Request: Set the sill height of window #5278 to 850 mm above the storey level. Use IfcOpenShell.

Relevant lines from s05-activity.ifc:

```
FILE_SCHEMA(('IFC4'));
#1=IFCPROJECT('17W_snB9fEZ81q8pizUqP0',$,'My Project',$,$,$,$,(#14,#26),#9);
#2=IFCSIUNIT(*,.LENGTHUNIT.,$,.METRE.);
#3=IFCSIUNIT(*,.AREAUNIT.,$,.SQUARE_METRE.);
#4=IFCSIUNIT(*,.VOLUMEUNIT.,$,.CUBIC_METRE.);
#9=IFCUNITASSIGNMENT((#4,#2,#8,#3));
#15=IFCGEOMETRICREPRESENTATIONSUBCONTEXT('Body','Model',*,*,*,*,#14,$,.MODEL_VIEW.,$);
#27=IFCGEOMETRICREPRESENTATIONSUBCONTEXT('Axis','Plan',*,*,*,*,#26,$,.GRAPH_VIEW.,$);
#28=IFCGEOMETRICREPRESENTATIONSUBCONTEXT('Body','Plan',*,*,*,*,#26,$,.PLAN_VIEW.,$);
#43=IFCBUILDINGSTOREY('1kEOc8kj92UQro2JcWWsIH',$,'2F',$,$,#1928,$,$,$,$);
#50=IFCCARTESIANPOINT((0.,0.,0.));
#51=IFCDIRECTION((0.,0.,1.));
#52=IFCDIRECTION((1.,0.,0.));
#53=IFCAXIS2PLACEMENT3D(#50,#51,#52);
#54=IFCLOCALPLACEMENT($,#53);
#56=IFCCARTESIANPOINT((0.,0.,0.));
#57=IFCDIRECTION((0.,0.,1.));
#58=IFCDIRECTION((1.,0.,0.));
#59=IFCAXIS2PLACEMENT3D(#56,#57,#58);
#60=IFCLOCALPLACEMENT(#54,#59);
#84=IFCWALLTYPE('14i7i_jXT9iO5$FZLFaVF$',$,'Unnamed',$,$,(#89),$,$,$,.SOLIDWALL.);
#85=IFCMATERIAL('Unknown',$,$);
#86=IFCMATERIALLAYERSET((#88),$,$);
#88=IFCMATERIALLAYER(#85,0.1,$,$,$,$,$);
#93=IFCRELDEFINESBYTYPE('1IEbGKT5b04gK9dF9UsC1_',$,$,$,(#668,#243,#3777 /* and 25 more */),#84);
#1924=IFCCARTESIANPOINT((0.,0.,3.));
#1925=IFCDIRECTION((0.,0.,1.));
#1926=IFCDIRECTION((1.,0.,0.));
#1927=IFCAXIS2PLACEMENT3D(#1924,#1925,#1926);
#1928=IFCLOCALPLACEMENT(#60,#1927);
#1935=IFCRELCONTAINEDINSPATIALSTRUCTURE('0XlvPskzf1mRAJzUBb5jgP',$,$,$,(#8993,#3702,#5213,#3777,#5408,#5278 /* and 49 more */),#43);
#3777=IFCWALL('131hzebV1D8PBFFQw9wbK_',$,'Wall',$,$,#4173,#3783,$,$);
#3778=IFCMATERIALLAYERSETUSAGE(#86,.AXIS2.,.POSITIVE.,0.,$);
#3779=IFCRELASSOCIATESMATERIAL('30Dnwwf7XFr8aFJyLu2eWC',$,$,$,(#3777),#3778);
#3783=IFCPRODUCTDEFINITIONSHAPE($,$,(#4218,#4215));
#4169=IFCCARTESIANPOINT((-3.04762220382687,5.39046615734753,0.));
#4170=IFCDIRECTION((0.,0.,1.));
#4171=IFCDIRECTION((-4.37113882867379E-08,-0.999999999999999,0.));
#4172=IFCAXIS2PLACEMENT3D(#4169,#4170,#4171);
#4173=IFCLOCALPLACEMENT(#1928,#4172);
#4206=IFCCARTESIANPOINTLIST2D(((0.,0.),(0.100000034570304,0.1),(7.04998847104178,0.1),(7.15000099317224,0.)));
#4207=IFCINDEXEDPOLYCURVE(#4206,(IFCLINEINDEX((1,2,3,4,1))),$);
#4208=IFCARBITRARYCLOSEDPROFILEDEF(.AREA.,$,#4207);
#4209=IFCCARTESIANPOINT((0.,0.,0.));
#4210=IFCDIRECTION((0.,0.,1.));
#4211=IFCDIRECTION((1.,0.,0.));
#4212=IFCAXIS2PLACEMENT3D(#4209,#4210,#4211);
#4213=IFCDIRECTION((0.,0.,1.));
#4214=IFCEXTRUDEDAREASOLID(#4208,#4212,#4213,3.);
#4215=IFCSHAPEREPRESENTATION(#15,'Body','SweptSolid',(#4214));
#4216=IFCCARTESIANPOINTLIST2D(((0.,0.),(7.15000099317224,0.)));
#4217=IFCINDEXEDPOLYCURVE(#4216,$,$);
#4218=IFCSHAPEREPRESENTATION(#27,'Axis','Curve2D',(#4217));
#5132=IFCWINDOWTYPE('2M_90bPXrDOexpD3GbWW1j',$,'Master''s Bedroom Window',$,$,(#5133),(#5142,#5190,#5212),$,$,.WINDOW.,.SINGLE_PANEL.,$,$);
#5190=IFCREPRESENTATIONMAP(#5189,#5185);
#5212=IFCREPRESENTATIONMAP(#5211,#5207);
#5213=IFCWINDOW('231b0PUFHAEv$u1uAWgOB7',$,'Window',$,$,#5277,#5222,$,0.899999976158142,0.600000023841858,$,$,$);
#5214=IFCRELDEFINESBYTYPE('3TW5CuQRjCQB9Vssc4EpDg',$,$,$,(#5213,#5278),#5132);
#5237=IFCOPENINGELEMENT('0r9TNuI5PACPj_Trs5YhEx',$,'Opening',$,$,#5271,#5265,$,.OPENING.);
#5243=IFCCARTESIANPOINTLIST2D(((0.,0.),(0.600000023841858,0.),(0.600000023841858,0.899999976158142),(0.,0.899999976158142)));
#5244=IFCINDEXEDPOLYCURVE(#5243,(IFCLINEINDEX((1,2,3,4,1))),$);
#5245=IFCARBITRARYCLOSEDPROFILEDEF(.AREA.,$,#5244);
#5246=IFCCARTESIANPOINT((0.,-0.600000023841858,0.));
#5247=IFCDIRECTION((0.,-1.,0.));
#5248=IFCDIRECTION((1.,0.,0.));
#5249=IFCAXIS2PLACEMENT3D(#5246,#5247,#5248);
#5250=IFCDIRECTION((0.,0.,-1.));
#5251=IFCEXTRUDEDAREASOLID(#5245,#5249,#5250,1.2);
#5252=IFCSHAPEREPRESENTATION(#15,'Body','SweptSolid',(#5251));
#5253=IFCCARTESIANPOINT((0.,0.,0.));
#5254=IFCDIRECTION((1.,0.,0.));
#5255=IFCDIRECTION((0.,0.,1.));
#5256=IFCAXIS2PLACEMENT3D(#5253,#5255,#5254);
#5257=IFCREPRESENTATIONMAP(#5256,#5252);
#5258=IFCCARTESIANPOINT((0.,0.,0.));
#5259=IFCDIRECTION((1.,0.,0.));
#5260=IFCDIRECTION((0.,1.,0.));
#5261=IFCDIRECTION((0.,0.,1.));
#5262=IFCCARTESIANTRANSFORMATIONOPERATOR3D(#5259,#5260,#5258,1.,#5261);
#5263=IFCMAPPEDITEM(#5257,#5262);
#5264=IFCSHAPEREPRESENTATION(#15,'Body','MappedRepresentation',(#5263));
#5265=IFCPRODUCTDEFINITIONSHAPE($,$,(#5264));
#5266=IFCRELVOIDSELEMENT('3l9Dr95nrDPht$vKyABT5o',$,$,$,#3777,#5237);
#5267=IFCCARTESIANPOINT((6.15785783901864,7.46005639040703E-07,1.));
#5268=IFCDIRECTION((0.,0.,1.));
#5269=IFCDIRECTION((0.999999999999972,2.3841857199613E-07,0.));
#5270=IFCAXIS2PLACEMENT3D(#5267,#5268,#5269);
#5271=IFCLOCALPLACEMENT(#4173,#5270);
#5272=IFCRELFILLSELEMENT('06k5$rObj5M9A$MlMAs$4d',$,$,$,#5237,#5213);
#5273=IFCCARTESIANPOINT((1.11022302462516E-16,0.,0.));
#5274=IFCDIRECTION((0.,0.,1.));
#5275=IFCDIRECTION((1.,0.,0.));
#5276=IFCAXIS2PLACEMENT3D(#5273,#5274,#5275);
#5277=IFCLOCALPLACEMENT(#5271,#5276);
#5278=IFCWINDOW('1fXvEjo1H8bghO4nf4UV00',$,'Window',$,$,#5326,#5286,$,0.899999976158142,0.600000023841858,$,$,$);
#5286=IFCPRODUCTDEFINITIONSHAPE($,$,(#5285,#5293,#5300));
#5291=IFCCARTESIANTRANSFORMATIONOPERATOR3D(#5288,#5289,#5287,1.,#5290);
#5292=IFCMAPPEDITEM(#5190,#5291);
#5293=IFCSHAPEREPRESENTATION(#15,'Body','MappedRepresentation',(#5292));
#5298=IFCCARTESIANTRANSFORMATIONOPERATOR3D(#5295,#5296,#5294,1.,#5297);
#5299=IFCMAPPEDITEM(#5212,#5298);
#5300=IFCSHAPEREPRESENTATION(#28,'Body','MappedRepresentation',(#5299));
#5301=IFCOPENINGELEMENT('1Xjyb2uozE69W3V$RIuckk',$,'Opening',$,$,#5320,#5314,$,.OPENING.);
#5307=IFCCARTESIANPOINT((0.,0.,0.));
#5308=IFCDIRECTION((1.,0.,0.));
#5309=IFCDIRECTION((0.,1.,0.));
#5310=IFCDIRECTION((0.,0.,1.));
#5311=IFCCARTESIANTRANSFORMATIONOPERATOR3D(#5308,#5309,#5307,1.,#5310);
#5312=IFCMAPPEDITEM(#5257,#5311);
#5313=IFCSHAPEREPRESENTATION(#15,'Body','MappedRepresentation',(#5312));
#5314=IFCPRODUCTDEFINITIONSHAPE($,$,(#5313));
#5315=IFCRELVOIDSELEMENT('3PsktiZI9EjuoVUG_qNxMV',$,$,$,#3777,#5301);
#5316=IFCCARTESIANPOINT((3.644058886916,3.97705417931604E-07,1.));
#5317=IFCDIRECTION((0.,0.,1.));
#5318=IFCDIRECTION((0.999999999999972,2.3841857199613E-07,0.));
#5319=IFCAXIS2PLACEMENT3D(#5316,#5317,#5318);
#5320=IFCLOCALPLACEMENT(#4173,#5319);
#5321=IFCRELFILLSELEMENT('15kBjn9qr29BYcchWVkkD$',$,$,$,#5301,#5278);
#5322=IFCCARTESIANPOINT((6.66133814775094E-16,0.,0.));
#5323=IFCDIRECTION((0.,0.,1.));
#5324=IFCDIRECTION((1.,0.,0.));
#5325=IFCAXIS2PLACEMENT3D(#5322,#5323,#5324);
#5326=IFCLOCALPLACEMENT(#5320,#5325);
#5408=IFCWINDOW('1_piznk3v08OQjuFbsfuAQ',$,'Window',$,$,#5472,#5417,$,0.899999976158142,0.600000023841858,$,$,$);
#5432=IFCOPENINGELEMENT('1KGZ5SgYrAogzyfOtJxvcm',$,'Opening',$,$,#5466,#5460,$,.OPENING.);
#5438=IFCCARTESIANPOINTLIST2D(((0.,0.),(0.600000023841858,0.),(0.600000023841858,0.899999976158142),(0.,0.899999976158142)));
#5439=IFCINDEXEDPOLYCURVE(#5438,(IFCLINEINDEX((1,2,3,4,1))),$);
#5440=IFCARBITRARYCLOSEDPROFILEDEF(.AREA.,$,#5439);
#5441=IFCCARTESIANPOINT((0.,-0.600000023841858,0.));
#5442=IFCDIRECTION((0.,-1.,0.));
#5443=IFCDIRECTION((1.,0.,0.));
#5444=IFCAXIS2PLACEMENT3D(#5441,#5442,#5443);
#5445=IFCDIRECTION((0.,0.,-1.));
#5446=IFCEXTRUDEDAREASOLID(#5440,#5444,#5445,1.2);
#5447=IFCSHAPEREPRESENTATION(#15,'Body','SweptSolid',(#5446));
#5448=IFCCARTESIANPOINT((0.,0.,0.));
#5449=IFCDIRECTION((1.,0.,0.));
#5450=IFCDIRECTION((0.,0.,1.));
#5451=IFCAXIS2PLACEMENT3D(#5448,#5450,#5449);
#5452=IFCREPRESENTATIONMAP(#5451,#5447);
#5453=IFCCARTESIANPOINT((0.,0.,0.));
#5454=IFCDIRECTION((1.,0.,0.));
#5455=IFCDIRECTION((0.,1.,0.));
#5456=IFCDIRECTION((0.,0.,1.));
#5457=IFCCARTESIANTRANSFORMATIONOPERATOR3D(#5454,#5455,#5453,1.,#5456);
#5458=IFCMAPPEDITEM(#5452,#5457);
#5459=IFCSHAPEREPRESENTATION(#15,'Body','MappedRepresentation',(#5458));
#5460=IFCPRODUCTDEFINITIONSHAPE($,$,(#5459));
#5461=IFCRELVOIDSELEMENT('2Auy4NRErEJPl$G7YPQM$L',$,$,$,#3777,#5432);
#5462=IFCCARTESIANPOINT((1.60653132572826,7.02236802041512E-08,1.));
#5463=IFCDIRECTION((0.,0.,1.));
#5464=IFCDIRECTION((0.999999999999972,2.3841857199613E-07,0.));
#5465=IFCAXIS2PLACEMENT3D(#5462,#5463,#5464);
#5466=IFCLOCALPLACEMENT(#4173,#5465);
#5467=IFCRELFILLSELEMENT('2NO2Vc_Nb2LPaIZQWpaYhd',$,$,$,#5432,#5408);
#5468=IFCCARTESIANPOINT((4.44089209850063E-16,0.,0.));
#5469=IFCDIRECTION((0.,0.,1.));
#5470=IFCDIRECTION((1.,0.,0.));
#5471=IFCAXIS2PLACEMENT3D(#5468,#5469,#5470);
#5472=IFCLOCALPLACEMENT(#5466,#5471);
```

```python
import numpy as np
import ifcopenshell
import ifcopenshell.api.geometry
import ifcopenshell.geom
import ifcopenshell.util.element
import ifcopenshell.util.placement
import ifcopenshell.util.shape
import ifcopenshell.util.unit

model = ifcopenshell.open("s05-activity.ifc")
unit_scale = ifcopenshell.util.unit.calculate_unit_scale(model)

window = model.by_id(5278)
opening = window.FillsVoids[0].RelatingOpeningElement
storey = ifcopenshell.util.element.get_container(window, ifc_class="IfcBuildingStorey")
level = ifcopenshell.util.placement.get_local_placement(storey.ObjectPlacement)[2, 3]

# The opening's origin need not be at the sill, so measure its lowest point.
shape = ifcopenshell.geom.create_shape(ifcopenshell.geom.settings(), opening)
bottom = ifcopenshell.util.shape.get_shape_bottom_elevation(shape, shape.geometry) / unit_scale
dz = level + 0.85 / unit_scale - bottom

shift = np.array([0.0, 0.0, dz])
# The window is placed relative to its opening, so it follows when the opening moves.
matrix = ifcopenshell.util.placement.get_local_placement(opening.ObjectPlacement)
matrix[:3, 3] += shift
ifcopenshell.api.geometry.edit_object_placement(
    model, product=opening, matrix=matrix, is_si=False, should_transform_children=True
)

print(f"moved by {dz * unit_scale:+.3f} m")

model.write("s05-activity-out.ifc")
```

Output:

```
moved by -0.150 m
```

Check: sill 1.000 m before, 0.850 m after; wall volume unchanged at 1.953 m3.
